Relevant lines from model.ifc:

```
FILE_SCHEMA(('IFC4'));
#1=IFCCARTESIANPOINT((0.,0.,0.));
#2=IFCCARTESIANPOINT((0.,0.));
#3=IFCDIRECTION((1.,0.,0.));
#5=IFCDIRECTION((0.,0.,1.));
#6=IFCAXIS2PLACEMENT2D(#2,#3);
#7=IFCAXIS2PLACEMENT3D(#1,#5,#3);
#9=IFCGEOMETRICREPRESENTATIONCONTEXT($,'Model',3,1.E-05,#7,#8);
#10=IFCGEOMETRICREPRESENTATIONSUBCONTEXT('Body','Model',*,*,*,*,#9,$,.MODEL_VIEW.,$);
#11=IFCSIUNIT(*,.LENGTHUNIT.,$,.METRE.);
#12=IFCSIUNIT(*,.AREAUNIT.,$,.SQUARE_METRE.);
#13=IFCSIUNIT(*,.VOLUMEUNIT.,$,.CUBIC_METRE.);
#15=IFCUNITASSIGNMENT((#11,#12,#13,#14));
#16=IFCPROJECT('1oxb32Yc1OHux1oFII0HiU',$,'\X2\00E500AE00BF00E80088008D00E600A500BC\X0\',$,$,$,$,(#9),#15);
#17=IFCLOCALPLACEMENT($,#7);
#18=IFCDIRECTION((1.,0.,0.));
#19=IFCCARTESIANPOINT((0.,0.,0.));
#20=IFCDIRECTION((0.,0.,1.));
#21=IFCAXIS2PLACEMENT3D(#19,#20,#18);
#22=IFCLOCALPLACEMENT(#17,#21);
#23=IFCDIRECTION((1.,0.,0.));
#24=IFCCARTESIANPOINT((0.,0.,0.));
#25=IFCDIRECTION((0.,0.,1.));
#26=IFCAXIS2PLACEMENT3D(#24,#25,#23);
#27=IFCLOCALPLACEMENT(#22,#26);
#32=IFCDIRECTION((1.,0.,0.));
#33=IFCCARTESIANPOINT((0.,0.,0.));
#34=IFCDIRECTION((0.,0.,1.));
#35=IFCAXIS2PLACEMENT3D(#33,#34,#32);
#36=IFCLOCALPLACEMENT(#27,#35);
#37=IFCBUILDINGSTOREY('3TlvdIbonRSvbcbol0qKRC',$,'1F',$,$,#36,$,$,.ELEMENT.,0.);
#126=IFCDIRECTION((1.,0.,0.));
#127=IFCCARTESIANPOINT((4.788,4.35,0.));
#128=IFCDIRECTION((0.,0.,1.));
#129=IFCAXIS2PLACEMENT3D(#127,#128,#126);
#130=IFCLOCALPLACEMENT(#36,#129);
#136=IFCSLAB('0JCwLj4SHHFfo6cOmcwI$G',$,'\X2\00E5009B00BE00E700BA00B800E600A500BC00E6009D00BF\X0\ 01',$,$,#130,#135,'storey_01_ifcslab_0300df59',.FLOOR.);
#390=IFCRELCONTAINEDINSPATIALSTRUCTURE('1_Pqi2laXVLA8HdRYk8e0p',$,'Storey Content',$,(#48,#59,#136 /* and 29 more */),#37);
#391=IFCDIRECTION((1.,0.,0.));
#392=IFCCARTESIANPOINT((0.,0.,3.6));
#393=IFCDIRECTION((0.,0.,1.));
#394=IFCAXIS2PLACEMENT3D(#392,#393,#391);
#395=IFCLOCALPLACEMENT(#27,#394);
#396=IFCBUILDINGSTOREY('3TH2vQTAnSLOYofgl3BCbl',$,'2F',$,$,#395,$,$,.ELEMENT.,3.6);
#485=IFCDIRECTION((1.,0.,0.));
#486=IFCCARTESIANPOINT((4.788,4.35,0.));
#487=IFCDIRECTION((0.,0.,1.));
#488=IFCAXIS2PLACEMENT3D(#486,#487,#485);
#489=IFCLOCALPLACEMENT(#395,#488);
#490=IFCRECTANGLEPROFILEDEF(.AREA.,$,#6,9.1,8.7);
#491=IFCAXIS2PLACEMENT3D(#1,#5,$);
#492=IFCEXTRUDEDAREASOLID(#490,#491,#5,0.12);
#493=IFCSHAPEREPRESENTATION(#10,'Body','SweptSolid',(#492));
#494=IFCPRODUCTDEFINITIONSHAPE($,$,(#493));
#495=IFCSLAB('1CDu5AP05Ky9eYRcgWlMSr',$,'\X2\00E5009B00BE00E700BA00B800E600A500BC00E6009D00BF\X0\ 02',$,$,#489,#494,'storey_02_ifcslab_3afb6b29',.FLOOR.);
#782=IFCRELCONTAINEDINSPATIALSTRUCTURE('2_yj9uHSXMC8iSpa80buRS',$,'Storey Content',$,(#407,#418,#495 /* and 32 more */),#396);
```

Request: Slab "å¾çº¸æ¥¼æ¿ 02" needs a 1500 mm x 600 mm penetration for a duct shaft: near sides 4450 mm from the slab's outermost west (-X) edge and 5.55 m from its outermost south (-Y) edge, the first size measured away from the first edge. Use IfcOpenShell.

```python
import numpy as np
import ifcopenshell
import ifcopenshell.api.feature
import ifcopenshell.api.geometry
import ifcopenshell.api.root
import ifcopenshell.geom
import ifcopenshell.util.placement
import ifcopenshell.util.representation
import ifcopenshell.util.shape
import ifcopenshell.util.unit

model = ifcopenshell.open("model.ifc")
unit_scale = ifcopenshell.util.unit.calculate_unit_scale(model)
settings = ifcopenshell.geom.settings()


def volume(element):
    """Net volume in cubic metres, openings subtracted."""
    shape = ifcopenshell.geom.create_shape(settings, element)
    return ifcopenshell.util.shape.get_volume(shape.geometry)


slab = model.by_guid("1CDu5AP05Ky9eYRcgWlMSr")
before = volume(slab)

# Extent in the slab's own axes, in metres. The edges named are its -X and -Y sides.
slab_shape = ifcopenshell.geom.create_shape(settings, slab)
vertices = ifcopenshell.util.shape.get_vertices(slab_shape.geometry)
x_min, y_min, bottom = vertices.min(axis=0)
top = vertices[:, 2].max()

opening = ifcopenshell.api.root.create_entity(model, ifc_class="IfcOpeningElement", name="Duct shaft opening", predefined_type="OPENING")
context = ifcopenshell.util.representation.get_context(model, "Model", "Body", "MODEL_VIEW")
width, depth = 1.5, 0.6
outline = [(0.0, 0.0), (width, 0.0), (width, depth), (0.0, depth), (0.0, 0.0)]
# Overshoot both faces by 50 mm so the cut is clean.
shape = ifcopenshell.api.geometry.add_slab_representation(
    model, context=context, depth=top - bottom + 0.1, polyline=outline
)
ifcopenshell.api.geometry.assign_representation(model, product=opening, representation=shape)

matrix = ifcopenshell.util.placement.get_local_placement(slab.ObjectPlacement)
matrix[:, 3] = matrix @ np.append(np.array([x_min + 4.45, y_min + 5.55, bottom - 0.05]) / unit_scale, 1.0)
ifcopenshell.api.geometry.edit_object_placement(model, product=opening, matrix=matrix, is_si=False)
ifcopenshell.api.feature.add_feature(model, feature=opening, element=slab)

after = volume(slab)

print(f"slab volume {before:.3f} -> {after:.3f} m3")

model.write("model_rev.ifc")
```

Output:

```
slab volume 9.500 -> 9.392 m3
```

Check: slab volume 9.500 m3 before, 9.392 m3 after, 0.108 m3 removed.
